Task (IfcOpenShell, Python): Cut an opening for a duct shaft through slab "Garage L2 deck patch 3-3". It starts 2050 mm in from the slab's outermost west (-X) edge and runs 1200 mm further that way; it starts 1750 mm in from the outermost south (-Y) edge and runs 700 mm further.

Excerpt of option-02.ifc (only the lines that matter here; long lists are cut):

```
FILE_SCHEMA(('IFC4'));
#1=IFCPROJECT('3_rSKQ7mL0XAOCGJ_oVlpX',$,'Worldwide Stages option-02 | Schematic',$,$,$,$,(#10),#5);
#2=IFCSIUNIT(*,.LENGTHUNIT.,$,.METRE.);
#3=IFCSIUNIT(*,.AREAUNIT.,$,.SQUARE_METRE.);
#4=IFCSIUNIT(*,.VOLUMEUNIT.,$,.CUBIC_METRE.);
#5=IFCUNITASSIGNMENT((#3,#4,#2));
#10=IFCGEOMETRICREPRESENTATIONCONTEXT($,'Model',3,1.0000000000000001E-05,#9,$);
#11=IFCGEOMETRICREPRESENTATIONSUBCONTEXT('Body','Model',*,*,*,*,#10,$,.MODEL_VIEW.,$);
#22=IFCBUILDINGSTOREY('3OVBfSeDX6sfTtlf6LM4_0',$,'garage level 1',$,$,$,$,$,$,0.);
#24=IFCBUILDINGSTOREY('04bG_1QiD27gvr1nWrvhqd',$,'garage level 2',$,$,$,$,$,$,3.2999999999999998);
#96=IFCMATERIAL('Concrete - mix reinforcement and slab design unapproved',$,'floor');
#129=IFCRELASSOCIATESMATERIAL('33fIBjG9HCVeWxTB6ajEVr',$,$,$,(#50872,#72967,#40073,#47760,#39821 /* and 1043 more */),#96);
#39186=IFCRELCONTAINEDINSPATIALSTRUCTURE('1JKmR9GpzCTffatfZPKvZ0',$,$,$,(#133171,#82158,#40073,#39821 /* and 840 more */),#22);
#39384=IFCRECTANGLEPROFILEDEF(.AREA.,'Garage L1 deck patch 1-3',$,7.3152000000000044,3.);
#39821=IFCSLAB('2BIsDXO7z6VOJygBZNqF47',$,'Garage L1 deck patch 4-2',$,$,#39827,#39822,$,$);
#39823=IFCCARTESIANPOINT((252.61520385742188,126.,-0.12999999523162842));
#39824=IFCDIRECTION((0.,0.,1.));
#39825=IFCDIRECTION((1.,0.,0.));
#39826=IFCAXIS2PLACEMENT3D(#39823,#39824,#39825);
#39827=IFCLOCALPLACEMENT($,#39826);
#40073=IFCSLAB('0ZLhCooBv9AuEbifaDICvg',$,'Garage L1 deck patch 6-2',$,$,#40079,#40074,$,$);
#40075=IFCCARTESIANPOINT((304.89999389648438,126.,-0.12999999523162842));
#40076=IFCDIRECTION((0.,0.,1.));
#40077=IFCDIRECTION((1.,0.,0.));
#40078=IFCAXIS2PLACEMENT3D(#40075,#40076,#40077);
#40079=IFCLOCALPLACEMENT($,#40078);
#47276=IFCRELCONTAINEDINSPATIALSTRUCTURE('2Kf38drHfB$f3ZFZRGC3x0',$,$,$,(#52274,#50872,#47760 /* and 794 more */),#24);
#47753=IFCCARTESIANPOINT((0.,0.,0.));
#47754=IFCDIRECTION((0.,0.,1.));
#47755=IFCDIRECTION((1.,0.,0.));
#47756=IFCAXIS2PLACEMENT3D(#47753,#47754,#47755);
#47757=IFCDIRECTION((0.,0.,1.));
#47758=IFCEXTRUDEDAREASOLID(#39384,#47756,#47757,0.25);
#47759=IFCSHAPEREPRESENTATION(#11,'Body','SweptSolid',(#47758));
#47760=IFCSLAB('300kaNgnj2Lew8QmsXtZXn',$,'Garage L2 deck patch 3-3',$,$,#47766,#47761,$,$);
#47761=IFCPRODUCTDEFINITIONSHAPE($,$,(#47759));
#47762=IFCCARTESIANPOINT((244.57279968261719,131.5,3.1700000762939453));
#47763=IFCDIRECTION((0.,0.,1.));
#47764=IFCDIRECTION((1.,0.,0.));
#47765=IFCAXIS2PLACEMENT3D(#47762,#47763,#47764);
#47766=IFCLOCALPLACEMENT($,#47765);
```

```python
import numpy as np
import ifcopenshell
import ifcopenshell.api.feature
import ifcopenshell.api.geometry
import ifcopenshell.api.root
import ifcopenshell.geom
import ifcopenshell.util.placement
import ifcopenshell.util.representation
import ifcopenshell.util.shape
import ifcopenshell.util.unit

model = ifcopenshell.open("option-02.ifc")
unit_scale = ifcopenshell.util.unit.calculate_unit_scale(model)
settings = ifcopenshell.geom.settings()


def volume(element):
    """Net volume in cubic metres, openings subtracted."""
    shape = ifcopenshell.geom.create_shape(settings, element)
    return ifcopenshell.util.shape.get_volume(shape.geometry)


slab = model.by_id(47760)
before = volume(slab)

# Extent in the slab's own axes, in metres. The edges named are its -X and -Y sides.
slab_shape = ifcopenshell.geom.create_shape(settings, slab)
vertices = ifcopenshell.util.shape.get_vertices(slab_shape.geometry)
x_min, y_min, bottom = vertices.min(axis=0)
top = vertices[:, 2].max()

opening = ifcopenshell.api.root.create_entity(model, ifc_class="IfcOpeningElement", name="Duct shaft opening", predefined_type="OPENING")
context = ifcopenshell.util.representation.get_context(model, "Model", "Body", "MODEL_VIEW")
width, depth = 1.2, 0.7
outline = [(0.0, 0.0), (width, 0.0), (width, depth), (0.0, depth), (0.0, 0.0)]
# Overshoot both faces by 50 mm so the cut is clean.
shape = ifcopenshell.api.geometry.add_slab_representation(
    model, context=context, depth=top - bottom + 0.1, polyline=outline
)
ifcopenshell.api.geometry.assign_representation(model, product=opening, representation=shape)

matrix = ifcopenshell.util.placement.get_local_placement(slab.ObjectPlacement)
matrix[:, 3] = matrix @ np.append(np.array([x_min + 2.05, y_min + 1.75, bottom - 0.05]) / unit_scale, 1.0)
ifcopenshell.api.geometry.edit_object_placement(model, product=opening, matrix=matrix, is_si=False)
ifcopenshell.api.feature.add_feature(model, feature=opening, element=slab)

after = volume(slab)

print(f"slab volume {before:.3f} -> {after:.3f} m3")

model.write("option-02_rev.ifc")
```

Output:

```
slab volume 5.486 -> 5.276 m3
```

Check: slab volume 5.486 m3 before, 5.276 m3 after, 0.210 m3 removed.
